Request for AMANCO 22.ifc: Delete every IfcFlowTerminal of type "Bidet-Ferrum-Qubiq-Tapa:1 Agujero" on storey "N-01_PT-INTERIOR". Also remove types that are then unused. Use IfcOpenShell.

First a look at what the model holds.

```python
import ifcopenshell
import ifcopenshell.util.element

model = ifcopenshell.open("AMANCO 22.ifc")
print(model.schema)
storey = next(s for s in model.by_type("IfcBuildingStorey") if s.Name == "N-01_PT-INTERIOR")
terminals = [e for e in ifcopenshell.util.element.get_decomposition(storey) if e.is_a("IfcFlowTerminal")]
seen = {}
for e in terminals:
    element_type = ifcopenshell.util.element.get_type(e)
    name = element_type.Name if element_type not in (None, e) else None
    seen[name] = seen.get(name, 0) + 1
for name, count in sorted(seen.items(), key=str):
    print(count, "x", name)
```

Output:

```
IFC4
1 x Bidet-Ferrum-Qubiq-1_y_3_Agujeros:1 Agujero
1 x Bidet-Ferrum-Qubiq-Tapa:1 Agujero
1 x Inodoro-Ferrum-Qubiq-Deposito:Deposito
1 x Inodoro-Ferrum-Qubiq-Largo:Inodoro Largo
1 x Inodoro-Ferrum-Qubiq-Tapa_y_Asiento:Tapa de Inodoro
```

```python
import ifcopenshell
import ifcopenshell.api.root
import ifcopenshell.util.element

model = ifcopenshell.open("AMANCO 22.ifc")

storey = next(s for s in model.by_type("IfcBuildingStorey") if s.Name == "N-01_PT-INTERIOR")
terminals = [e for e in ifcopenshell.util.element.get_decomposition(storey) if e.is_a("IfcFlowTerminal")]
targets = [e for e in terminals if (t := ifcopenshell.util.element.get_type(e)) not in (None, e) and t.Name == "Bidet-Ferrum-Qubiq-Tapa:1 Agujero"]
types = {ifcopenshell.util.element.get_type(e) for e in targets} - {None, *targets}

for e in targets:
    ifcopenshell.api.root.remove_product(model, product=e)
print(len(targets), "removed")

unused = [t for t in types if not ifcopenshell.util.element.get_types(t)]
for t in unused:
    ifcopenshell.api.root.remove_product(model, product=t)
print(len(unused), "unused types removed")

model.write("AMANCO 22_updated.ifc")
```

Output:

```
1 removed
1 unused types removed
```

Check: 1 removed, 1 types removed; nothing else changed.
